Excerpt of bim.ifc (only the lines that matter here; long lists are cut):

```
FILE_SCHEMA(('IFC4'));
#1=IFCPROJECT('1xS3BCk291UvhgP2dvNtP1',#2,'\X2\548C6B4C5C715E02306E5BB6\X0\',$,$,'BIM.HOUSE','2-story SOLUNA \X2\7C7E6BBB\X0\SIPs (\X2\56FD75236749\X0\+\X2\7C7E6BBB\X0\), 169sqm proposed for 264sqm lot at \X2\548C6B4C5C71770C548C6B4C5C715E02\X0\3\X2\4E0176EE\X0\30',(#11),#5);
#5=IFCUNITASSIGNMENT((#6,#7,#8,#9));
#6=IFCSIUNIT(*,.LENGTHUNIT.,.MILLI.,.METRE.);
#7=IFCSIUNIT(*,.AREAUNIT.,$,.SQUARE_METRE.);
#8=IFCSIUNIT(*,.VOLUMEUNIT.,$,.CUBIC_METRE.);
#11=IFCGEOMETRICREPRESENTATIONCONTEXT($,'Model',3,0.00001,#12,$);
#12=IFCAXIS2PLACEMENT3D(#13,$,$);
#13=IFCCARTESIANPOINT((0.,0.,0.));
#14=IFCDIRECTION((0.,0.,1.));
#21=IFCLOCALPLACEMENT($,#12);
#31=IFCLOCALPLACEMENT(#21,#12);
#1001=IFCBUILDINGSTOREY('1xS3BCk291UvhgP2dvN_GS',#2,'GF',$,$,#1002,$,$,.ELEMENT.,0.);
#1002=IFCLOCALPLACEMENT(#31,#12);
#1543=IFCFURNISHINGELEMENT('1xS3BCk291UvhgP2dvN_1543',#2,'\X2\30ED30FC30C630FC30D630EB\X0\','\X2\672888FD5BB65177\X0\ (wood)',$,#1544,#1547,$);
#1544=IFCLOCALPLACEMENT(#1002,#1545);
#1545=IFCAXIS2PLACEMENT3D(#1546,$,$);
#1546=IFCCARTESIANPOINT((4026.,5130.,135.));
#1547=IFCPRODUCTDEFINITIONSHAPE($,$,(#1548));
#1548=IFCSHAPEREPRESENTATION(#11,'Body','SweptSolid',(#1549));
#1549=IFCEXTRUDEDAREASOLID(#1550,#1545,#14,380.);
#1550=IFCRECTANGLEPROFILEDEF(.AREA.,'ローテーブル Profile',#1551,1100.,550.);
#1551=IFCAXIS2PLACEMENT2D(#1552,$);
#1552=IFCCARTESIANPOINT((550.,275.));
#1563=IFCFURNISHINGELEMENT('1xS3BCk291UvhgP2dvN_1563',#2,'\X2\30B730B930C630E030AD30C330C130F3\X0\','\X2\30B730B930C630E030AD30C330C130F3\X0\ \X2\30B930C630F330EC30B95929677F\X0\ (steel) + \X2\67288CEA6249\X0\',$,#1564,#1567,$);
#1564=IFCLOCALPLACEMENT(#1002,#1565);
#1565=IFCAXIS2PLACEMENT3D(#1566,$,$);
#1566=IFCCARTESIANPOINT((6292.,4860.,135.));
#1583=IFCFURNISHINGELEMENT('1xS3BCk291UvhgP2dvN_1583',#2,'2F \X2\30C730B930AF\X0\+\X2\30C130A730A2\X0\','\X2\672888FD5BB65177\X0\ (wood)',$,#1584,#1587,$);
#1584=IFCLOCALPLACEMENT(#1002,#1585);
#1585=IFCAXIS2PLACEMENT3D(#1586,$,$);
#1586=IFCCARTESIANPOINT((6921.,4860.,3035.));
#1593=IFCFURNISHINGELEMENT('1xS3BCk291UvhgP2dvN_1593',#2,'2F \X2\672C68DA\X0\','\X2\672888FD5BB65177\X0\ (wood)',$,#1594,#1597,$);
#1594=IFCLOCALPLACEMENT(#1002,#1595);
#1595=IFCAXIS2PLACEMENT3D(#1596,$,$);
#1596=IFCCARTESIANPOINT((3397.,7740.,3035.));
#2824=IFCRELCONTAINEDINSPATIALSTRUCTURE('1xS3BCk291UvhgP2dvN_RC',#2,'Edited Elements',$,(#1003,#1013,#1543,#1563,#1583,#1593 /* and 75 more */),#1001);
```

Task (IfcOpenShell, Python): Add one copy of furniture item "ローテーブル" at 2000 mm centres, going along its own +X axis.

```python
import ifcopenshell
import ifcopenshell.api.geometry
import ifcopenshell.api.root
import ifcopenshell.util.element
import ifcopenshell.util.placement
import ifcopenshell.util.unit

model = ifcopenshell.open("bim.ifc")
unit_scale = ifcopenshell.util.unit.calculate_unit_scale(model)


def reuse_history(source, copy):
    """copy_class also copies each property set's owner history, people and application; keep the originals."""
    for rel in copy.IsDefinedBy:
        if rel.is_a("IfcRelDefinesByProperties") and (history := rel.RelatingPropertyDefinition.OwnerHistory):
            rel.RelatingPropertyDefinition.OwnerHistory = source.OwnerHistory
            ifcopenshell.util.element.remove_deep2(model, history)


source = model.by_id(1543)
base = ifcopenshell.util.placement.get_local_placement(source.ObjectPlacement)
step = base[:3, 0] * 2 / unit_scale

for i in range(1, 2):
    copy = ifcopenshell.api.root.copy_class(model, product=source)
    copy.Representation = ifcopenshell.util.element.copy_deep(
        model, source.Representation, exclude=["IfcGeometricRepresentationContext", "IfcRepresentationMap"]
    )
    reuse_history(source, copy)
    matrix = base.copy()
    matrix[:3, 3] += i * step
    print("added at", matrix[:3, 3].round(3) + 0.0)
    ifcopenshell.api.geometry.edit_object_placement(model, product=copy, matrix=matrix, is_si=False)

model.write("bim_edited.ifc")
```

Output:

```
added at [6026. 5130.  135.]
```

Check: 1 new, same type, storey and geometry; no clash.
